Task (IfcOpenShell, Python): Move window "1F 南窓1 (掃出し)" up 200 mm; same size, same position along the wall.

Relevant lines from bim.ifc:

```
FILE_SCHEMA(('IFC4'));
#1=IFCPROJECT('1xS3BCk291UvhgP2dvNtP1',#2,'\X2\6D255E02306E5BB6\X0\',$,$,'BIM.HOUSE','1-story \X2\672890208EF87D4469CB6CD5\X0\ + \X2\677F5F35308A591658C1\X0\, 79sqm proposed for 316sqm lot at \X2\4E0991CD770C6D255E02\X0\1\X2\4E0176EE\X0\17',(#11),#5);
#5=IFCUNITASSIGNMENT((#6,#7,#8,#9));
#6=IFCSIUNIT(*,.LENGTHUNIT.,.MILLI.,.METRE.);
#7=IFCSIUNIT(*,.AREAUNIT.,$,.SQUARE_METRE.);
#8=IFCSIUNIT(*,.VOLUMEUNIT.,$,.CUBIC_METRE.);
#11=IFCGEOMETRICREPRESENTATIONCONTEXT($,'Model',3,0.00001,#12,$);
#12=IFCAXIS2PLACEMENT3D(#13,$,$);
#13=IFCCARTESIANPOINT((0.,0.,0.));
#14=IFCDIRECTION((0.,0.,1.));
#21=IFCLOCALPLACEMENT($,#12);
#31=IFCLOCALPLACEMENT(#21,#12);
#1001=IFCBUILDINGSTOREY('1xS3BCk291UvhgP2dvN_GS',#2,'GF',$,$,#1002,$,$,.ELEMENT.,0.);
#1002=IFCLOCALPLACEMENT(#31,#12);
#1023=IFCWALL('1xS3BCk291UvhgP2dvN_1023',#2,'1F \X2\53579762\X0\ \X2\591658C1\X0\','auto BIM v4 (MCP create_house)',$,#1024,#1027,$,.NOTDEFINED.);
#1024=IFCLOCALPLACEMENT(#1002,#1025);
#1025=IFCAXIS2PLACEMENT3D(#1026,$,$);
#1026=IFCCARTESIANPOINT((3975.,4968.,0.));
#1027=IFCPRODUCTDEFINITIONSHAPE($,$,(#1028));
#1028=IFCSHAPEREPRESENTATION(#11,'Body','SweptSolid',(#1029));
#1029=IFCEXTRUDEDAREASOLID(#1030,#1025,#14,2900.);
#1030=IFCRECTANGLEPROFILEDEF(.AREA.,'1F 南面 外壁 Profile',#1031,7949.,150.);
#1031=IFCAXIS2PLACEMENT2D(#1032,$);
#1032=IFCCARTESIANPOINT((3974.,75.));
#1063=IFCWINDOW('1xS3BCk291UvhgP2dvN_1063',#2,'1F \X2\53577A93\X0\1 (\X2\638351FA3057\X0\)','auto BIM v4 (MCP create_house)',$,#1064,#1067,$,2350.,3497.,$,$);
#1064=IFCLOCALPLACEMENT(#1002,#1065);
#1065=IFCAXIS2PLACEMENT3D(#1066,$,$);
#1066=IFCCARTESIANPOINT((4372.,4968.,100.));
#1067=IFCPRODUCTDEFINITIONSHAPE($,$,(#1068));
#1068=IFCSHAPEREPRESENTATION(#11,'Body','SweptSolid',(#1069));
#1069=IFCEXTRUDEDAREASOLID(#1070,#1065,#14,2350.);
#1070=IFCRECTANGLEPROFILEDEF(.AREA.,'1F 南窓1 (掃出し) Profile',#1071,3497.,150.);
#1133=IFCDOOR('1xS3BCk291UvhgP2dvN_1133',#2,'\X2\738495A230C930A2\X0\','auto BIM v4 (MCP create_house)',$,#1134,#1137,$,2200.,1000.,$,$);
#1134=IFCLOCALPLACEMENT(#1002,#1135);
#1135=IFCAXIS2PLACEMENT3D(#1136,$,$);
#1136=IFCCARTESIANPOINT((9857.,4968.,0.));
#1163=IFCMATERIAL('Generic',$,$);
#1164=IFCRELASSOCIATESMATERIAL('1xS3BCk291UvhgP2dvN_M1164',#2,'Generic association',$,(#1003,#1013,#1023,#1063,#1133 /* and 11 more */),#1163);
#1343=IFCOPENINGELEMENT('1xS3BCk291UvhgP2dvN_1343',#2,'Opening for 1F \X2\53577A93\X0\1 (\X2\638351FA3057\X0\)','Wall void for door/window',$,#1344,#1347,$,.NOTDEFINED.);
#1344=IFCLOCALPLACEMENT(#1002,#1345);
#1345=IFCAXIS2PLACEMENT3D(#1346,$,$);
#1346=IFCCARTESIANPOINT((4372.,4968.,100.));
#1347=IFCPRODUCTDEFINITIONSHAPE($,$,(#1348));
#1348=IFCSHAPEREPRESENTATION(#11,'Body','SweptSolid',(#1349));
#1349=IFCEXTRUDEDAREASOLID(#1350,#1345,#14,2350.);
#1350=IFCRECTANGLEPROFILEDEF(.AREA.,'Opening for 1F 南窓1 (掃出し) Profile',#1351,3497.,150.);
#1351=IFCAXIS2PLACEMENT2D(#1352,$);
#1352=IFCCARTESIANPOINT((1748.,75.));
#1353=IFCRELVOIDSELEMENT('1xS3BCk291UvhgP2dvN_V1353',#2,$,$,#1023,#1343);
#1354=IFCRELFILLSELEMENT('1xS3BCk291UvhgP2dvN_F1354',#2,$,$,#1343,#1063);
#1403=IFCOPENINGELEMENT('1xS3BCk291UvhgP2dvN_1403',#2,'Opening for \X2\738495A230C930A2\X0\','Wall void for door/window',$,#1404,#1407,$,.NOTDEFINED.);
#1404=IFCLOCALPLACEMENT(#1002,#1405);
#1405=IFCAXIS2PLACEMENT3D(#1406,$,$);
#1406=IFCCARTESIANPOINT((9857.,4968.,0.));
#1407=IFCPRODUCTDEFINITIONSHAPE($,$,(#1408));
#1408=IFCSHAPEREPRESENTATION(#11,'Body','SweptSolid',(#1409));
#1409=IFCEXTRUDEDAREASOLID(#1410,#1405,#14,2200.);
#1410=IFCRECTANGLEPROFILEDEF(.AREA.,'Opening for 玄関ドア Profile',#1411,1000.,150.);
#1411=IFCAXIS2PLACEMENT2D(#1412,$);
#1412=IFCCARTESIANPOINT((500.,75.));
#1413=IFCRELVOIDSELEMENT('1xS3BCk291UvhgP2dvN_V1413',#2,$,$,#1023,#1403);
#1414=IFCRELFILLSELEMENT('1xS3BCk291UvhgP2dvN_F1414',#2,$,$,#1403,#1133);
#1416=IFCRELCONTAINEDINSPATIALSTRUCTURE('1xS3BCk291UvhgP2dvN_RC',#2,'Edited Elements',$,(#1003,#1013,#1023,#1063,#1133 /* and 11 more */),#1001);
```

```python
import numpy as np
import ifcopenshell
import ifcopenshell.api.geometry
import ifcopenshell.util.placement
import ifcopenshell.util.unit

model = ifcopenshell.open("bim.ifc")
unit_scale = ifcopenshell.util.unit.calculate_unit_scale(model)

window = model.by_guid("1xS3BCk291UvhgP2dvN_1063")
opening = window.FillsVoids[0].RelatingOpeningElement
dz = 0.2 / unit_scale

shift = np.array([0.0, 0.0, dz])
# The window is not placed relative to its opening, so move both.
for product in (opening, window):
    matrix = ifcopenshell.util.placement.get_local_placement(product.ObjectPlacement)
    matrix[:3, 3] += shift
    ifcopenshell.api.geometry.edit_object_placement(model, product=product, matrix=matrix, is_si=False)

print(f"moved by {dz * unit_scale:+.3f} m")

model.write("bim-out.ifc")
```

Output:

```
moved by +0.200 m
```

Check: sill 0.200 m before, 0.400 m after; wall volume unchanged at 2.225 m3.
